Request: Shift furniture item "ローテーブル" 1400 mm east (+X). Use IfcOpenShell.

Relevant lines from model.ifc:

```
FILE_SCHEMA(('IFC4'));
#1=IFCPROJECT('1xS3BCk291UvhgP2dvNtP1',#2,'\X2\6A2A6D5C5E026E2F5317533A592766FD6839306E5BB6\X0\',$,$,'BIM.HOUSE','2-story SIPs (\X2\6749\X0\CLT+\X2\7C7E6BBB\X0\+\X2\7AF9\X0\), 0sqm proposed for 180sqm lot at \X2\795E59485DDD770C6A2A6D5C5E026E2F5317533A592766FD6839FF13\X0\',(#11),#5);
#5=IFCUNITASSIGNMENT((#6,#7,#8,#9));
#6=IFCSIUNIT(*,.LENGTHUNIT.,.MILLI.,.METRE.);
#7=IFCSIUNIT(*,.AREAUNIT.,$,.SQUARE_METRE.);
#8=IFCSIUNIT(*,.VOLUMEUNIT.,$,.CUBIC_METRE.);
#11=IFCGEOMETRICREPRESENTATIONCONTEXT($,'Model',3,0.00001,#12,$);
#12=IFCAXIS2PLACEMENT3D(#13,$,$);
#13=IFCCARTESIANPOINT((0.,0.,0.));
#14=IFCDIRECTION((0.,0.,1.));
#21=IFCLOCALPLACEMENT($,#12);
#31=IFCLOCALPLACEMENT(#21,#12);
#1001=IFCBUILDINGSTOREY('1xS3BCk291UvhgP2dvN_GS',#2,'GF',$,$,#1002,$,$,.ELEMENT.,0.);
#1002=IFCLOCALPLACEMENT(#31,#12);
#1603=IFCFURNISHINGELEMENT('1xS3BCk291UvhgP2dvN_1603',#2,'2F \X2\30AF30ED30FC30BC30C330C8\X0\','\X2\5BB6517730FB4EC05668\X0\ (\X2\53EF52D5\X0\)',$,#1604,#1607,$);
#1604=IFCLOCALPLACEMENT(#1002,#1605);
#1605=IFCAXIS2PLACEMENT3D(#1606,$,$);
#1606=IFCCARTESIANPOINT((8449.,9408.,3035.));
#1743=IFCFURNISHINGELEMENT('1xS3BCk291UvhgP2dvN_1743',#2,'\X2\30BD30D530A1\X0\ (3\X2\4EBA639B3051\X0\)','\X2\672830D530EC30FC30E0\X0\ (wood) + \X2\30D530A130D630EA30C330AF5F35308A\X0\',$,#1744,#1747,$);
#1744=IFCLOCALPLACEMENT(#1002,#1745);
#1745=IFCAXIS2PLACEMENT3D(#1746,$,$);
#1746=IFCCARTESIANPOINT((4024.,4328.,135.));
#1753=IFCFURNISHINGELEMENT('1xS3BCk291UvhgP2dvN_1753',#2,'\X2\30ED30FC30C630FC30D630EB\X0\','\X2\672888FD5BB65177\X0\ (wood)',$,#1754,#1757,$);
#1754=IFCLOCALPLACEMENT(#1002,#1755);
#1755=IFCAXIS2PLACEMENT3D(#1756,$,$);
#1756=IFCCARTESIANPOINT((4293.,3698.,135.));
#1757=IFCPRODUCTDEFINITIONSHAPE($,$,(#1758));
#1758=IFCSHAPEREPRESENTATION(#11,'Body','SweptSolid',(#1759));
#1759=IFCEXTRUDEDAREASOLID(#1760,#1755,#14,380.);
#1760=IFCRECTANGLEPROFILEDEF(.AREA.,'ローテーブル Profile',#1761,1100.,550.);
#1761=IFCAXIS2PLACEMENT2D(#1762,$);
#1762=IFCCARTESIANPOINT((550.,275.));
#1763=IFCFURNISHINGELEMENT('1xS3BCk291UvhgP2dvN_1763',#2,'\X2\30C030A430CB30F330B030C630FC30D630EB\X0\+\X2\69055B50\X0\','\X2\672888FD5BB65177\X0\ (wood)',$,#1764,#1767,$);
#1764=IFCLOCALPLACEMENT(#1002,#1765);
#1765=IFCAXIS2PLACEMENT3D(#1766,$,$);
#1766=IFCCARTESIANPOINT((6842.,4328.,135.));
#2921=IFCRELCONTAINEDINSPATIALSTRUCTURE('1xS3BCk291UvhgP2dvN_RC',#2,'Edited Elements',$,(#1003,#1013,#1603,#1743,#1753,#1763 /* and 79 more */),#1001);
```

```python
import ifcopenshell
import ifcopenshell.api.geometry
import ifcopenshell.util.placement
import ifcopenshell.util.unit

model = ifcopenshell.open("model.ifc")
unit_scale = ifcopenshell.util.unit.calculate_unit_scale(model)

item = model.by_guid("1xS3BCk291UvhgP2dvN_1753")
matrix = ifcopenshell.util.placement.get_local_placement(item.ObjectPlacement)
matrix[0, 3] += 1.4 / unit_scale
ifcopenshell.api.geometry.edit_object_placement(model, product=item, matrix=matrix, is_si=False)

print(ifcopenshell.util.placement.get_local_placement(item.ObjectPlacement).round(3) + 0.0)

model.write("model_rev.ifc")
```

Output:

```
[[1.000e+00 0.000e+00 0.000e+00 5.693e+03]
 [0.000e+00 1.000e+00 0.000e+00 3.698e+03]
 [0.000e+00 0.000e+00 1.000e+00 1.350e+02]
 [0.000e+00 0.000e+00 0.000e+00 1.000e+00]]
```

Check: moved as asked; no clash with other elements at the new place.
